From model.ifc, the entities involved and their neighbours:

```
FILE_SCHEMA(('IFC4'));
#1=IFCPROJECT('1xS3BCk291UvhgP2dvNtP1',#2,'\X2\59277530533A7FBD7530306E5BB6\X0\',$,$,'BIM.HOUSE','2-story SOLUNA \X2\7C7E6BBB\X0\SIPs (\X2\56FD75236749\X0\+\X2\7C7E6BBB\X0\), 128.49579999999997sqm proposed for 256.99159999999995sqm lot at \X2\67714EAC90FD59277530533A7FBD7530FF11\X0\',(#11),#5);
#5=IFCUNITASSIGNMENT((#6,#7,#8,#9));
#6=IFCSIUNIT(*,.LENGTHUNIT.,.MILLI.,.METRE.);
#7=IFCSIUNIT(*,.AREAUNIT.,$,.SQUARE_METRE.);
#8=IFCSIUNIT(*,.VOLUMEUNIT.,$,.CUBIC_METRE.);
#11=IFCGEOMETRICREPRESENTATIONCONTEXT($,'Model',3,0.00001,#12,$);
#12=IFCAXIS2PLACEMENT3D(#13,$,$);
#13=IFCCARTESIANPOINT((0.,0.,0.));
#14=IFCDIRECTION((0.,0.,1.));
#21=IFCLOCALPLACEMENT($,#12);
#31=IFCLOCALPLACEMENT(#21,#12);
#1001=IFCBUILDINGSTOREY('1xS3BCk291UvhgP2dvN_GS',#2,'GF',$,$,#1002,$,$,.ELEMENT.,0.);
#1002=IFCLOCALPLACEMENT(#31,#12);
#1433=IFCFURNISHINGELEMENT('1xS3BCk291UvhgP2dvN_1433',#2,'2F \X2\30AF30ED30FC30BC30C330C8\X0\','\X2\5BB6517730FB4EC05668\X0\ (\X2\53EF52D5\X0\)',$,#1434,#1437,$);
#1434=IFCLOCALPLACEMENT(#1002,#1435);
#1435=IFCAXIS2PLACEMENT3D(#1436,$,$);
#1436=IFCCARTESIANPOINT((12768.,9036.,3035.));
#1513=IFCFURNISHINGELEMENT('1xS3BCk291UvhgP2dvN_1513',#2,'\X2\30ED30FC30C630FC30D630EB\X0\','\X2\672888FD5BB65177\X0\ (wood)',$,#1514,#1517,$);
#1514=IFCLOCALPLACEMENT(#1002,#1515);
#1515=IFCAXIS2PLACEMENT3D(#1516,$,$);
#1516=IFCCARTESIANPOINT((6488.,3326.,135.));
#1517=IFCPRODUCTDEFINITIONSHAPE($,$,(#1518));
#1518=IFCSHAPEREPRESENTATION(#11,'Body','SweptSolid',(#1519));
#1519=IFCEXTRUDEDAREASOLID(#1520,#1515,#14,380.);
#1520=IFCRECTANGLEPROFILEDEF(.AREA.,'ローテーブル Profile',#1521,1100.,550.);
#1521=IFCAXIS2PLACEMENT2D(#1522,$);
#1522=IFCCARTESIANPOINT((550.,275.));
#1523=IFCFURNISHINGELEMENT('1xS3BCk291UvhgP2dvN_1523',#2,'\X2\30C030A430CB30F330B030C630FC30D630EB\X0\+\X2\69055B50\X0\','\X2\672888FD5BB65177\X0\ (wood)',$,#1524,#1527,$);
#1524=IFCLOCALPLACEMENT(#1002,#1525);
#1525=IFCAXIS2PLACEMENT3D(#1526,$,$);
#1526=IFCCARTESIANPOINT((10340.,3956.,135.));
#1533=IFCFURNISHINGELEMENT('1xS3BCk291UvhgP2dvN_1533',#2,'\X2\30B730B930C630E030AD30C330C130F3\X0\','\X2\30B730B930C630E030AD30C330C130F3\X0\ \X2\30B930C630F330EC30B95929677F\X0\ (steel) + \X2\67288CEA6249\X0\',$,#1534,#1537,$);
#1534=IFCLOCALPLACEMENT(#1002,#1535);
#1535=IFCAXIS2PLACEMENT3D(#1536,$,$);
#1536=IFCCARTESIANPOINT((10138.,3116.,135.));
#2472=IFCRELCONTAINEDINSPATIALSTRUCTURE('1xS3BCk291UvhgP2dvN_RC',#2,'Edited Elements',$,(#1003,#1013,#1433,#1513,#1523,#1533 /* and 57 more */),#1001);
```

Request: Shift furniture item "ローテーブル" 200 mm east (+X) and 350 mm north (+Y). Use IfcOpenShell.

```python
import ifcopenshell
import ifcopenshell.api.geometry
import ifcopenshell.util.placement

model = ifcopenshell.open("model.ifc")

item = model.by_guid("1xS3BCk291UvhgP2dvN_1513")
matrix = ifcopenshell.util.placement.get_local_placement(item.ObjectPlacement)
matrix[0, 3] += 200.0
matrix[1, 3] += 350.0
ifcopenshell.api.geometry.edit_object_placement(model, product=item, matrix=matrix, is_si=False)

print(ifcopenshell.util.placement.get_local_placement(item.ObjectPlacement).round(3) + 0.0)

model.write("model_v2.ifc")
```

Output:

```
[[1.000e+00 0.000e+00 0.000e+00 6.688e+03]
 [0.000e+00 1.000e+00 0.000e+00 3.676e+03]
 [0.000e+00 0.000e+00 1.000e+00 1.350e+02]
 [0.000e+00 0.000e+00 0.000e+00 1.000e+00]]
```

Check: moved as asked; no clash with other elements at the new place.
